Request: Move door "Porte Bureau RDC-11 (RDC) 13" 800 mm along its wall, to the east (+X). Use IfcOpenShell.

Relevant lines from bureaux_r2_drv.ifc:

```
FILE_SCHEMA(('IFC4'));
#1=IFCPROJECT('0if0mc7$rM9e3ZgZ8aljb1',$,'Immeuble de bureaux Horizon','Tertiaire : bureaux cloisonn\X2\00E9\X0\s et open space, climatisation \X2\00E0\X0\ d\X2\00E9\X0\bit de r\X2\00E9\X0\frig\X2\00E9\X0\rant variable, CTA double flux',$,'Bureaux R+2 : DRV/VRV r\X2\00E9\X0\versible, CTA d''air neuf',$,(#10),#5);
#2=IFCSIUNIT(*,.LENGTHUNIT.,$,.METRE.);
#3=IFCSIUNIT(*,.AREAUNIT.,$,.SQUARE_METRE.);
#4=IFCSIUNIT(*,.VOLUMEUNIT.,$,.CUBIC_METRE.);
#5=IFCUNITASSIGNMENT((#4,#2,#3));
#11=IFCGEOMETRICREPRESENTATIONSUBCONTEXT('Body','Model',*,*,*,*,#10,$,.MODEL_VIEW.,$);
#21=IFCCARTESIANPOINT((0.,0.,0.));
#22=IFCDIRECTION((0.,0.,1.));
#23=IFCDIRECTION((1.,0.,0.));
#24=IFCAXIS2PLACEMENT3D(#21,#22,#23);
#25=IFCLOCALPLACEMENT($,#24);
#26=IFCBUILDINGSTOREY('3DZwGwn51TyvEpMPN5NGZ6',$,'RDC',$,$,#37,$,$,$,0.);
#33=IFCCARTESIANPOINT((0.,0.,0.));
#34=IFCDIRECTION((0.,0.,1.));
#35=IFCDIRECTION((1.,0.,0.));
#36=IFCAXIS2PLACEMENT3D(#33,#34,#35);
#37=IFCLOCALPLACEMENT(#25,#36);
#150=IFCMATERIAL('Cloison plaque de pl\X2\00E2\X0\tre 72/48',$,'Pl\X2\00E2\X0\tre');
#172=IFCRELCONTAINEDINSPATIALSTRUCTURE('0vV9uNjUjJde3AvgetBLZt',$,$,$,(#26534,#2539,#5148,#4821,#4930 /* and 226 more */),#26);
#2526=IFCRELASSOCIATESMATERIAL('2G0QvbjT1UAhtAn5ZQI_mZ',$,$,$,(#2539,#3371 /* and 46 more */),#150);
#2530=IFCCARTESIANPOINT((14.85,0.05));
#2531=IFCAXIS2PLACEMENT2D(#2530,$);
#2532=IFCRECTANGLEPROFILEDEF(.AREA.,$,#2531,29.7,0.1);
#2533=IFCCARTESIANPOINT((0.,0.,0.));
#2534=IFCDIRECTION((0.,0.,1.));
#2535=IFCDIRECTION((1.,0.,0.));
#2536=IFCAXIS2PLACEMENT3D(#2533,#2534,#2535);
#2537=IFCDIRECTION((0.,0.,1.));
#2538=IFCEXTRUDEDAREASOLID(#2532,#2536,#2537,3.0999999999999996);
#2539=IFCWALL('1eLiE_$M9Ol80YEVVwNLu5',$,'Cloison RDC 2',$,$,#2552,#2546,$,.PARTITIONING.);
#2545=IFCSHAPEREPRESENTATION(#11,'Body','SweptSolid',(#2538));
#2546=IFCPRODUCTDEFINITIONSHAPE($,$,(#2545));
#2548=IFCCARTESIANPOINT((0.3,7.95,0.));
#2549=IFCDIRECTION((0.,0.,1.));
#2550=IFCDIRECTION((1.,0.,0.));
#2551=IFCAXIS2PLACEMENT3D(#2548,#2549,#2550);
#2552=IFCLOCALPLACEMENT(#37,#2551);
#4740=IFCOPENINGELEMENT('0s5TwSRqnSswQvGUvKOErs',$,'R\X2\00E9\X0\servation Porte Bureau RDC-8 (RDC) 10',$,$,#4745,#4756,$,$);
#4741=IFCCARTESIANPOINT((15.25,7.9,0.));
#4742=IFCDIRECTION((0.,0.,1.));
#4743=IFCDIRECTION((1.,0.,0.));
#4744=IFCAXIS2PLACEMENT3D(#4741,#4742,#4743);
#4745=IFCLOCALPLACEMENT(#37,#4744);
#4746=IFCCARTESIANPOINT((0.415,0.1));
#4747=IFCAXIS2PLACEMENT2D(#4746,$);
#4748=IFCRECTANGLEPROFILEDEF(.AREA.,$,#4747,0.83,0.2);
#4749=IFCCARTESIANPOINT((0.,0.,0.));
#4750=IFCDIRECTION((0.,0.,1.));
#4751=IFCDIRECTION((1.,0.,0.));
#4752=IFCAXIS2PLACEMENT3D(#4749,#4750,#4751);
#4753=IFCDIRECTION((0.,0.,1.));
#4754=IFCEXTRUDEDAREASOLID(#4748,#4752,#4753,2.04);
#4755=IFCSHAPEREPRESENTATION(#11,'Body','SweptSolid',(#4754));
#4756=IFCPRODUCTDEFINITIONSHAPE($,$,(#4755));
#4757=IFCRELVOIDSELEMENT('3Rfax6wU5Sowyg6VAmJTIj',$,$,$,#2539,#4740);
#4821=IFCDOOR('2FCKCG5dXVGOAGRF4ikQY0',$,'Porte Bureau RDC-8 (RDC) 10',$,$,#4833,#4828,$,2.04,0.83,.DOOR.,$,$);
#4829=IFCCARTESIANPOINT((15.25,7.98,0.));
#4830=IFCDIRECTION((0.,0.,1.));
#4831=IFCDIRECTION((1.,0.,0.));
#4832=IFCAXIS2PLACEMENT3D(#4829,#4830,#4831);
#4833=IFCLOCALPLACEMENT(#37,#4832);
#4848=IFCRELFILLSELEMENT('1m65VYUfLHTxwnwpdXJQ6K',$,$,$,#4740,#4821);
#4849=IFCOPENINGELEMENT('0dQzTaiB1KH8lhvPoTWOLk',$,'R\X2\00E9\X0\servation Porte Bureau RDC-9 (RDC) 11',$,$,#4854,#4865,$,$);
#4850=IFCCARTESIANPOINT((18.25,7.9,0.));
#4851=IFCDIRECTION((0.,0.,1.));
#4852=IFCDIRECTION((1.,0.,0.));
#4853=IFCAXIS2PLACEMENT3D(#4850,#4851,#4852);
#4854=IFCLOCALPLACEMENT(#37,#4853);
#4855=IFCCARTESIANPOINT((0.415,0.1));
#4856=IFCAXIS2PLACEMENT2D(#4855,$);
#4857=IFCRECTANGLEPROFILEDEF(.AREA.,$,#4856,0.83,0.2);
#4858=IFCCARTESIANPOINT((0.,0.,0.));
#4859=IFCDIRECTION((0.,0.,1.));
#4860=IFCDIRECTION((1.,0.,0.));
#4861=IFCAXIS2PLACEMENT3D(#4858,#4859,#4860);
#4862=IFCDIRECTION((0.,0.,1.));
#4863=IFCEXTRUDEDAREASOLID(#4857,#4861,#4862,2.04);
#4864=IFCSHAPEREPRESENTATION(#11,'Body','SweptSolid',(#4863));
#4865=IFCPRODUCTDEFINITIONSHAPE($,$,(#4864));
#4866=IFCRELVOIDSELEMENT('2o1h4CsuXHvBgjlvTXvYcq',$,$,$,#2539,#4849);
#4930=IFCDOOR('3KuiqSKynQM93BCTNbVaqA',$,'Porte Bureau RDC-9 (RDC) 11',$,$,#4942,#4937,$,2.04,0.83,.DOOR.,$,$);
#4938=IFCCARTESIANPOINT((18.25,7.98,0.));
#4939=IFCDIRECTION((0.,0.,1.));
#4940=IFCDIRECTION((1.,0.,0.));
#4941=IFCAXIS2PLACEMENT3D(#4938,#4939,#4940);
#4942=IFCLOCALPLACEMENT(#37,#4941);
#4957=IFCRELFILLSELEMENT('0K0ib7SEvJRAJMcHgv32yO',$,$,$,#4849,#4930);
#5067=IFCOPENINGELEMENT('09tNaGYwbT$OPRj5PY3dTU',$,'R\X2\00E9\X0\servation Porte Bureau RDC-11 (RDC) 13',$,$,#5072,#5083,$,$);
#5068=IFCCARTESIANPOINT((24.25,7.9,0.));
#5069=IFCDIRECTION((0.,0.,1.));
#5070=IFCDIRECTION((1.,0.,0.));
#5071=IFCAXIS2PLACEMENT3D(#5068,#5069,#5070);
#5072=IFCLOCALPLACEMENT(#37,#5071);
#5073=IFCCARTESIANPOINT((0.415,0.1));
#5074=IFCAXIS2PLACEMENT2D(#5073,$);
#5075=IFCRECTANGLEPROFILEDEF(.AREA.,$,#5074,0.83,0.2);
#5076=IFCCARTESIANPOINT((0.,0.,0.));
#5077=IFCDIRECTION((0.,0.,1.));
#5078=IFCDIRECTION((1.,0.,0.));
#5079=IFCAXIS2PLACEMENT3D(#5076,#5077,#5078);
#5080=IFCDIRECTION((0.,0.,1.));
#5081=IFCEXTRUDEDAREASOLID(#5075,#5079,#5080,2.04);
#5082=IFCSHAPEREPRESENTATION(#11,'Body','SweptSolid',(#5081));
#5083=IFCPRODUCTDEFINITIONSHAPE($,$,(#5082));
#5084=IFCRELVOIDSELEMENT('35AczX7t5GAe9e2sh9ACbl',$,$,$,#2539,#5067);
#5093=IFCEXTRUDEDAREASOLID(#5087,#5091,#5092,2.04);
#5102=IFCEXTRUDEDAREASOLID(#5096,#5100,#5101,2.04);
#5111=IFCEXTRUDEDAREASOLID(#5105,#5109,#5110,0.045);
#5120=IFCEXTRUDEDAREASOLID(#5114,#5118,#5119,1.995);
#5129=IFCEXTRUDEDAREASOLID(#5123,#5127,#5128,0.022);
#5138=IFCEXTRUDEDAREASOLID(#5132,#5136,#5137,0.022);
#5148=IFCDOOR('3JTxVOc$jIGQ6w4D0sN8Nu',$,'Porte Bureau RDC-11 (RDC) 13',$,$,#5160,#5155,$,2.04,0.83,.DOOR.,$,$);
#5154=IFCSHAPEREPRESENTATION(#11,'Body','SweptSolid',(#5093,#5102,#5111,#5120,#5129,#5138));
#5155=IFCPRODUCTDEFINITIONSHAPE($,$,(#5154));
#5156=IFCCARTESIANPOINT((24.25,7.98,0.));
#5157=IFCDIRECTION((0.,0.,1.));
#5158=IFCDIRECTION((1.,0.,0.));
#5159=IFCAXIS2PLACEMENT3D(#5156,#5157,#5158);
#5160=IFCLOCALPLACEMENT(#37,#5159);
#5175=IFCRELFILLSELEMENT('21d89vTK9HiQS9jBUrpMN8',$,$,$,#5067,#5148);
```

```python
import ifcopenshell
import ifcopenshell.api.geometry
import ifcopenshell.util.placement

model = ifcopenshell.open("bureaux_r2_drv.ifc")

door = model.by_guid("3JTxVOc$jIGQ6w4D0sN8Nu")
opening = door.FillsVoids[0].RelatingOpeningElement
wall = opening.VoidsElements[0].RelatingBuildingElement

wall_matrix = ifcopenshell.util.placement.get_local_placement(wall.ObjectPlacement)
shift = wall_matrix[:3, 0] * 0.8
before = ifcopenshell.util.placement.get_local_placement(door.ObjectPlacement)[:3, 3].copy()

# The door is not placed relative to its opening, so move both.
for product in (opening, door):
    matrix = ifcopenshell.util.placement.get_local_placement(product.ObjectPlacement)
    matrix[:3, 3] += shift
    ifcopenshell.api.geometry.edit_object_placement(model, product=product, matrix=matrix, is_si=False)

after = ifcopenshell.util.placement.get_local_placement(door.ObjectPlacement)[:3, 3]
print("door moved by", (after - before).round(3) + 0.0)

model.write("bureaux_r2_drv_edited.ifc")
```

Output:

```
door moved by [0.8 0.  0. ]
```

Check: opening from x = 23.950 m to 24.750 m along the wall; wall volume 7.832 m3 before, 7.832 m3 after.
